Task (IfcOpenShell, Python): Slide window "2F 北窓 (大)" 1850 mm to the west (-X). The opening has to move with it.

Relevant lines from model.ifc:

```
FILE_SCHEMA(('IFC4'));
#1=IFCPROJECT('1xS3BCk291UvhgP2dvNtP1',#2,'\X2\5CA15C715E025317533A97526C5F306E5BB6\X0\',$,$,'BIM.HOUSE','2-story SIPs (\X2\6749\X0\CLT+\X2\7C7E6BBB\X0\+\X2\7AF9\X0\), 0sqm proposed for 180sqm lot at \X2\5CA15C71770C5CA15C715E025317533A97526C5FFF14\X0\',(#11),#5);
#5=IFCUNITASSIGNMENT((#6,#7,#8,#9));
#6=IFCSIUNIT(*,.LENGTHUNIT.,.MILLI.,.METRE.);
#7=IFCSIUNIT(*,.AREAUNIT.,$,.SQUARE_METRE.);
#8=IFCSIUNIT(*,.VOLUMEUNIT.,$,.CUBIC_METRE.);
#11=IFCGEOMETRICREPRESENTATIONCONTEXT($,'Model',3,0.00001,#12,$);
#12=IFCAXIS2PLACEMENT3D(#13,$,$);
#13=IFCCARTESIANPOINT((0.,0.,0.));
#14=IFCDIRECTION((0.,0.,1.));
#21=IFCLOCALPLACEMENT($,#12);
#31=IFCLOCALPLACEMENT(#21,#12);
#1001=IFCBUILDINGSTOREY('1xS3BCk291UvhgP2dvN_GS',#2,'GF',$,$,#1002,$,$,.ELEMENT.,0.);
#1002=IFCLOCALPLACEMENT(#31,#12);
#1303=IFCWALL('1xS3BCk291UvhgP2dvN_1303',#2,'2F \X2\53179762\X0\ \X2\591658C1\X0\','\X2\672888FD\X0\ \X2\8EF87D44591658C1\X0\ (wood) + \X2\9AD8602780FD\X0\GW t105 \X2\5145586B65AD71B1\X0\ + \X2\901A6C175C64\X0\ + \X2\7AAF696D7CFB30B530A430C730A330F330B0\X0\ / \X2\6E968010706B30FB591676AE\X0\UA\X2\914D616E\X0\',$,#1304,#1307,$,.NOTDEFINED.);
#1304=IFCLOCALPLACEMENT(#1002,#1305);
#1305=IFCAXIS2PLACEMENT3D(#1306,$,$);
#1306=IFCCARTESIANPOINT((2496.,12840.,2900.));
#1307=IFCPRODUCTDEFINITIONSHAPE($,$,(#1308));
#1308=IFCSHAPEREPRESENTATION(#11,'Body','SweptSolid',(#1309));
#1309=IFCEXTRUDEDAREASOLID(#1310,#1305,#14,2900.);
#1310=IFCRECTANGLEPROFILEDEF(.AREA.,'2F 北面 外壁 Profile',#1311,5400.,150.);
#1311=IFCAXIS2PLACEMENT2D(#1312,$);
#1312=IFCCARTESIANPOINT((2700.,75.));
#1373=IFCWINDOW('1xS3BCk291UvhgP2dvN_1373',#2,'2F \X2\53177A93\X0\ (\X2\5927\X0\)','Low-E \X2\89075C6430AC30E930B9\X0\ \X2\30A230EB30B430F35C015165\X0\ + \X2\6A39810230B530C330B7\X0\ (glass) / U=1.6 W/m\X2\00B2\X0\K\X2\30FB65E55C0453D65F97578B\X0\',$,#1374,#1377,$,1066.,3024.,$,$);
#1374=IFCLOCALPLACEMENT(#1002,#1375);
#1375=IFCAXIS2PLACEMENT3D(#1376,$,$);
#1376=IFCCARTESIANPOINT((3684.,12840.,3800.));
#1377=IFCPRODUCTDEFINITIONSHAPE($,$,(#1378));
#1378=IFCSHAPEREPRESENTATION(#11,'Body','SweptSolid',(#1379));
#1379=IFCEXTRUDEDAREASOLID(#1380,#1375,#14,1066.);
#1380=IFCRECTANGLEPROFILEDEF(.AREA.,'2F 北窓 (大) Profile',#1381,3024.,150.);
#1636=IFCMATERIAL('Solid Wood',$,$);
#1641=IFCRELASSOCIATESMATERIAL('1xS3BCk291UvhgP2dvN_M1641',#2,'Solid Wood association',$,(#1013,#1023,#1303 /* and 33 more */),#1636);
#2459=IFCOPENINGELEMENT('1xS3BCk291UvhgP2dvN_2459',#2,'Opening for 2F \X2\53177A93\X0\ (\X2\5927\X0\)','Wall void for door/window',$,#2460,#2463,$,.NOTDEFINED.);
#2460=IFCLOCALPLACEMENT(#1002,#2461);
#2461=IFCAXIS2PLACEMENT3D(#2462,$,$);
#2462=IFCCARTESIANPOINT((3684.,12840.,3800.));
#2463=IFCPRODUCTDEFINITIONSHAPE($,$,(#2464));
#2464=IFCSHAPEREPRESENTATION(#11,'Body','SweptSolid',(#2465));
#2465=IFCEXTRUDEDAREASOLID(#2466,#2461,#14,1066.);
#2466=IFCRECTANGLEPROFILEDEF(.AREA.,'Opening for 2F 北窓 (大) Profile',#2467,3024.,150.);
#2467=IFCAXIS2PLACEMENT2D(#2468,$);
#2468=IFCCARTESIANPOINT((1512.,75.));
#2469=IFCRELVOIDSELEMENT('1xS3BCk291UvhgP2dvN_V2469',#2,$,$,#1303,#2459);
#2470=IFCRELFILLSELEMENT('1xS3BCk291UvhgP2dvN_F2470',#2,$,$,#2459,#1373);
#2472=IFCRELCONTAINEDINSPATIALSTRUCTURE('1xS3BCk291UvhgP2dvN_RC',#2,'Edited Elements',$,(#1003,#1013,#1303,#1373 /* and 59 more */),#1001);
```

```python
import ifcopenshell
import ifcopenshell.api.geometry
import ifcopenshell.util.placement

model = ifcopenshell.open("model.ifc")

window = model.by_guid("1xS3BCk291UvhgP2dvN_1373")
opening = window.FillsVoids[0].RelatingOpeningElement
wall = opening.VoidsElements[0].RelatingBuildingElement

wall_matrix = ifcopenshell.util.placement.get_local_placement(wall.ObjectPlacement)
shift = wall_matrix[:3, 0] * -1850.0
before = ifcopenshell.util.placement.get_local_placement(window.ObjectPlacement)[:3, 3].copy()

# The window is not placed relative to its opening, so move both.
for product in (opening, window):
    matrix = ifcopenshell.util.placement.get_local_placement(product.ObjectPlacement)
    matrix[:3, 3] += shift
    ifcopenshell.api.geometry.edit_object_placement(model, product=product, matrix=matrix, is_si=False)

after = ifcopenshell.util.placement.get_local_placement(window.ObjectPlacement)[:3, 3]
print("window moved by", (after - before).round(3) + 0.0)

model.write("model_rev.ifc")
```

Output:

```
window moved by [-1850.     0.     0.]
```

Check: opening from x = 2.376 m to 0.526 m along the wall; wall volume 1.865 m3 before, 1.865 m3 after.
